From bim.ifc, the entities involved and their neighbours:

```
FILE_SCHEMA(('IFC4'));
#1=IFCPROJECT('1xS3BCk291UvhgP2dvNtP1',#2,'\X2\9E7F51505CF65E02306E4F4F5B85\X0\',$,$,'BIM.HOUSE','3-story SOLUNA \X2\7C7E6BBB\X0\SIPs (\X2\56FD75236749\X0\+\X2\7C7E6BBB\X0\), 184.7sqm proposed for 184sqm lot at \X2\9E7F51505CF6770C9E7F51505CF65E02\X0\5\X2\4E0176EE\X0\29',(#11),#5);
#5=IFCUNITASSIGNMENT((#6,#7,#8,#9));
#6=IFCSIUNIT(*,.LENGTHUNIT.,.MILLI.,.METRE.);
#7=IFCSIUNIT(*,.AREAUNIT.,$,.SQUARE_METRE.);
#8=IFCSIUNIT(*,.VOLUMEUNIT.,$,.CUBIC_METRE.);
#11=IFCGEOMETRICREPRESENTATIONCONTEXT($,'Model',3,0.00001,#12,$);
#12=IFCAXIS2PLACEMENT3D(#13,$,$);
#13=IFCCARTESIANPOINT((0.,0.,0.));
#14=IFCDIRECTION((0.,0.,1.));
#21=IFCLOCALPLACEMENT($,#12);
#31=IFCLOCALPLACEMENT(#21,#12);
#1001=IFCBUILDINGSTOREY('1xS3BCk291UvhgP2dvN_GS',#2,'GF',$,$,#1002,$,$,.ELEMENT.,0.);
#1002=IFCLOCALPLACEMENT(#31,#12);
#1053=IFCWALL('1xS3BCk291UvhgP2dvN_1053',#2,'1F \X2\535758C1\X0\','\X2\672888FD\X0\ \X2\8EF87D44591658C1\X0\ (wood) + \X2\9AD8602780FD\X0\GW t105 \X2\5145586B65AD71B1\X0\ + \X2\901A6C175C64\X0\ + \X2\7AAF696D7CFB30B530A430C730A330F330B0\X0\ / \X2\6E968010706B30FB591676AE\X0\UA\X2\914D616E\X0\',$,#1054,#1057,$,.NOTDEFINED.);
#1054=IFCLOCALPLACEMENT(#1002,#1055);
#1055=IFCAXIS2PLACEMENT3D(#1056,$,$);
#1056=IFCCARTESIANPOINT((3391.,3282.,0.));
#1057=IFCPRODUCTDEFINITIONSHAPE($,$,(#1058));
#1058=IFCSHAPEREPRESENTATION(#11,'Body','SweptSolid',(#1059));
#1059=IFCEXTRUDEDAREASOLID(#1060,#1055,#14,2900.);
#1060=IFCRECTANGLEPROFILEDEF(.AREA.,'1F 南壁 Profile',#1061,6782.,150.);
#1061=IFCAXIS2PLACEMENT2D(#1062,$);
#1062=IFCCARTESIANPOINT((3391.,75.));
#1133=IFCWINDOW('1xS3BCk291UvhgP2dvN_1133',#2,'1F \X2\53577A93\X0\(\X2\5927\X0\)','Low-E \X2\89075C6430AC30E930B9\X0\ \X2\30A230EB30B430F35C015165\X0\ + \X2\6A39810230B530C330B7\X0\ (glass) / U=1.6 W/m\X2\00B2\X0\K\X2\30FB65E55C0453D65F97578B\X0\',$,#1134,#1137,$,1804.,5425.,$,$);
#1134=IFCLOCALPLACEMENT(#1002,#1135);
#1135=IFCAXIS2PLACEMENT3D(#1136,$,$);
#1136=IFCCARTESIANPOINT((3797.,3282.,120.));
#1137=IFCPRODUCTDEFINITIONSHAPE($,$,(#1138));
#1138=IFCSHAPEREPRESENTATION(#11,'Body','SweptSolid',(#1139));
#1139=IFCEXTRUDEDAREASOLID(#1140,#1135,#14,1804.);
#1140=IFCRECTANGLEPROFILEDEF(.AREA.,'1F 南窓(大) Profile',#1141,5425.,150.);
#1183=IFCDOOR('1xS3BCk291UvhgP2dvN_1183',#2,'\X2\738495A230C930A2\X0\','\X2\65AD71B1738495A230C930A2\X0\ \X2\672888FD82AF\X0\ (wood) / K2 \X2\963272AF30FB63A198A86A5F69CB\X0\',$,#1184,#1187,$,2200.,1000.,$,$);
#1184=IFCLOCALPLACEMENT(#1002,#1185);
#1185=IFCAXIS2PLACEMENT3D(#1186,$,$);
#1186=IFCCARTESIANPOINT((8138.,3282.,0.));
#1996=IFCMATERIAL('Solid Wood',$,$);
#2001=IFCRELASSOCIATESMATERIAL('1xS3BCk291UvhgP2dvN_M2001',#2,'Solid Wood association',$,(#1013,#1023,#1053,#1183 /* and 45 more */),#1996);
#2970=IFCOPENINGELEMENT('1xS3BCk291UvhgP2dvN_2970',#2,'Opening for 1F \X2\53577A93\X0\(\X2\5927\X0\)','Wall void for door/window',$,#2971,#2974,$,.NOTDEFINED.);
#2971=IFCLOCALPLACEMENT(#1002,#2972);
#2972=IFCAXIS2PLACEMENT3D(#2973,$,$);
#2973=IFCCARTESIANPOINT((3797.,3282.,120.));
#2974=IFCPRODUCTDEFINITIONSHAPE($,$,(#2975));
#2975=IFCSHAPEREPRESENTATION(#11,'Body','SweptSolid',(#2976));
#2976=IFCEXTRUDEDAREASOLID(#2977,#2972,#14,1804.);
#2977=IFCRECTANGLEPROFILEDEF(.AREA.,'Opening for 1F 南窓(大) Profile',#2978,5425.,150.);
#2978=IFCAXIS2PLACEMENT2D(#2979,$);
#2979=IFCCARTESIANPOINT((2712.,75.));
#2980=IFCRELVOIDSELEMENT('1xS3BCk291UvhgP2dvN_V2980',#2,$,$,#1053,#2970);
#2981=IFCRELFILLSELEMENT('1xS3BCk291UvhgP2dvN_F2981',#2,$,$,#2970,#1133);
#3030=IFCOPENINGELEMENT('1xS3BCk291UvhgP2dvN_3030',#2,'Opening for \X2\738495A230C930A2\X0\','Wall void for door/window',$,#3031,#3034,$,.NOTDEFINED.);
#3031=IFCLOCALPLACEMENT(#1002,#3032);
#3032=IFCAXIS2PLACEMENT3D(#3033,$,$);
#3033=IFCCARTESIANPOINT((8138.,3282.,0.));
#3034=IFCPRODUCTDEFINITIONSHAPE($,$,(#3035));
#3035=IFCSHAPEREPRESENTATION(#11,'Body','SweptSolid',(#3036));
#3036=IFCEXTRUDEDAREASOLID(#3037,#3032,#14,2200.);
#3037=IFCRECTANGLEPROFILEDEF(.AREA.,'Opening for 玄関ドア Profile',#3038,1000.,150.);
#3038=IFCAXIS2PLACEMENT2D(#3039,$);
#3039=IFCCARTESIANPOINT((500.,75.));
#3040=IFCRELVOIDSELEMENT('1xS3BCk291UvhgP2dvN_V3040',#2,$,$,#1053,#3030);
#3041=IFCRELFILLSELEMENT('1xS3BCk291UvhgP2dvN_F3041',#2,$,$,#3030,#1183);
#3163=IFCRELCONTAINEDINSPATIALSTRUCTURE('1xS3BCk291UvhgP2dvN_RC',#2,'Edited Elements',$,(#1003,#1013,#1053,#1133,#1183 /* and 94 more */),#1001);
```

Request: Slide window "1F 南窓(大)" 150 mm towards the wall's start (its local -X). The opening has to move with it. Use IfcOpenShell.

```python
import ifcopenshell
import ifcopenshell.api.geometry
import ifcopenshell.util.placement

model = ifcopenshell.open("bim.ifc")

window = model.by_id(1133)
opening = window.FillsVoids[0].RelatingOpeningElement
wall = opening.VoidsElements[0].RelatingBuildingElement

wall_matrix = ifcopenshell.util.placement.get_local_placement(wall.ObjectPlacement)
shift = wall_matrix[:3, 0] * -150.0
before = ifcopenshell.util.placement.get_local_placement(window.ObjectPlacement)[:3, 3].copy()

# The window is not placed relative to its opening, so move both.
for product in (opening, window):
    matrix = ifcopenshell.util.placement.get_local_placement(product.ObjectPlacement)
    matrix[:3, 3] += shift
    ifcopenshell.api.geometry.edit_object_placement(model, product=product, matrix=matrix, is_si=False)

after = ifcopenshell.util.placement.get_local_placement(window.ObjectPlacement)[:3, 3]
print("window moved by", (after - before).round(3) + 0.0)

model.write("bim-out.ifc")
```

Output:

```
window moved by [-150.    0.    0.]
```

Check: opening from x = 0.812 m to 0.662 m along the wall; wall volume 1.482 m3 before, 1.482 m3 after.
